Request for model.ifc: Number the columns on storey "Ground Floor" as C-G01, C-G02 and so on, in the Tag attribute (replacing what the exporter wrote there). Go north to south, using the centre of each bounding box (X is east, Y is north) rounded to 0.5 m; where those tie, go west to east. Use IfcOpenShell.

First a look at what the model holds.

```python
import ifcopenshell
import ifcopenshell.util.element
import ifcopenshell.util.placement

model = ifcopenshell.open("model.ifc")
print(model.schema)
storey = next(s for s in model.by_type("IfcBuildingStorey") if s.Name == "Ground Floor")
columns = [e for e in ifcopenshell.util.element.get_decomposition(storey) if e.is_a("IfcColumn")]
for e in sorted(columns, key=lambda e: e.id()):
    origin = ifcopenshell.util.placement.get_local_placement(e.ObjectPlacement)[:3, 3]
    print(e.id(), e.Tag, e.Name, origin.round(2) + 0.0, sep=" | ")
```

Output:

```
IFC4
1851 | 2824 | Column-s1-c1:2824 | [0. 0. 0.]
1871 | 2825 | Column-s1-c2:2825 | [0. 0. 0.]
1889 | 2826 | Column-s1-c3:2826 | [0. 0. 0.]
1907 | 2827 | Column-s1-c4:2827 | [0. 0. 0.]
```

```python
import ifcopenshell
import ifcopenshell.geom
import ifcopenshell.util.element
import ifcopenshell.util.shape

model = ifcopenshell.open("model.ifc")
settings = ifcopenshell.geom.settings()
settings.set("use-world-coords", True)


def centre(element):
    shape = ifcopenshell.geom.create_shape(settings, element)
    return ifcopenshell.util.shape.get_bbox_centroid(shape.geometry)


storey = next(s for s in model.by_type("IfcBuildingStorey") if s.Name == "Ground Floor")
columns = [e for e in ifcopenshell.util.element.get_decomposition(storey) if e.is_a("IfcColumn")]

# Insertion points can sit at a corner or the storey origin, so sort by the geometry (in metres).
centres = {e: centre(e) for e in columns}
columns.sort(key=lambda e: (-round(centres[e][1] / 0.5), centres[e][0]))

for i, e in enumerate(columns, start=1):
    number = f"C-G{i:02d}"
    e.Tag = number
    print(e.id(), number)

model.write("model_v2.ifc")
```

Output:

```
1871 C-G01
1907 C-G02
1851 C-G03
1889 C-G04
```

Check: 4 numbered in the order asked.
